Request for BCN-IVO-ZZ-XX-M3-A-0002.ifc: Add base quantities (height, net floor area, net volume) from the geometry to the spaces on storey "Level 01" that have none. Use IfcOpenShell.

First a look at what the model holds.

```python
import ifcopenshell
import ifcopenshell.util.element
import ifcopenshell.util.unit

model = ifcopenshell.open("BCN-IVO-ZZ-XX-M3-A-0002.ifc")
print(model.schema)
for unit_type in ("LENGTHUNIT", "AREAUNIT", "VOLUMEUNIT"):
    print(unit_type, ifcopenshell.util.unit.calculate_unit_scale(model, unit_type))
storey = next(s for s in model.by_type("IfcBuildingStorey") if s.Name == "Level 01")
spaces = [e for e in ifcopenshell.util.element.get_decomposition(storey) if e.is_a("IfcSpace")]
for e in sorted(spaces, key=lambda e: e.id()):
    print(e.id(), e.is_a(), e.Name, list(ifcopenshell.util.element.get_psets(e, qtos_only=True)), sep=" | ")
```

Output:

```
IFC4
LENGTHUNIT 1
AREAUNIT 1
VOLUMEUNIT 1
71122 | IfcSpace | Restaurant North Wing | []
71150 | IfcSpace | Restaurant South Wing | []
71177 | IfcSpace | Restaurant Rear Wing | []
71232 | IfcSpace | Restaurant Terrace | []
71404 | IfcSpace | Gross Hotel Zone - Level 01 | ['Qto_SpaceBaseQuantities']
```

```python
import ifcopenshell
import ifcopenshell.api.pset
import ifcopenshell.geom
import ifcopenshell.util.element
import ifcopenshell.util.shape
import ifcopenshell.util.unit

model = ifcopenshell.open("BCN-IVO-ZZ-XX-M3-A-0002.ifc")
unit_scale = ifcopenshell.util.unit.calculate_unit_scale(model)
area_scale = ifcopenshell.util.unit.calculate_unit_scale(model, "AREAUNIT")
volume_scale = ifcopenshell.util.unit.calculate_unit_scale(model, "VOLUMEUNIT")
settings = ifcopenshell.geom.settings()

storey = next(s for s in model.by_type("IfcBuildingStorey") if s.Name == "Level 01")
spaces = [e for e in ifcopenshell.util.element.get_decomposition(storey) if e.is_a("IfcSpace")]

for e in sorted(spaces, key=lambda e: e.id()):
    if ifcopenshell.util.element.get_psets(e, qtos_only=True, should_inherit=False):
        continue
    # Geometry comes back in metres, in the element's own axes.
    shape = ifcopenshell.geom.create_shape(settings, e)
    values = {
        "Height": ifcopenshell.util.shape.get_z(shape.geometry) / unit_scale,
        "NetFloorArea": ifcopenshell.util.shape.get_footprint_area(shape.geometry) / area_scale,
        "NetVolume": ifcopenshell.util.shape.get_volume(shape.geometry) / volume_scale,
    }
    qto = ifcopenshell.api.pset.add_qto(model, product=e, name="Qto_SpaceBaseQuantities")
    ifcopenshell.api.pset.edit_qto(model, qto=qto, properties=values)
    print(e.id(), {k: round(v, 3) for k, v in values.items()})

model.write("BCN-IVO-ZZ-XX-M3-A-0002-out.ifc")
```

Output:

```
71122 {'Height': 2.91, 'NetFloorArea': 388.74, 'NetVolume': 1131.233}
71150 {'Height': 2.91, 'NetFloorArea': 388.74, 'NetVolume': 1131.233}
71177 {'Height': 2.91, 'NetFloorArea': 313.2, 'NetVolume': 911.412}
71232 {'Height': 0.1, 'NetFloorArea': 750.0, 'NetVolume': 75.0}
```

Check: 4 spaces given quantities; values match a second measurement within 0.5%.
